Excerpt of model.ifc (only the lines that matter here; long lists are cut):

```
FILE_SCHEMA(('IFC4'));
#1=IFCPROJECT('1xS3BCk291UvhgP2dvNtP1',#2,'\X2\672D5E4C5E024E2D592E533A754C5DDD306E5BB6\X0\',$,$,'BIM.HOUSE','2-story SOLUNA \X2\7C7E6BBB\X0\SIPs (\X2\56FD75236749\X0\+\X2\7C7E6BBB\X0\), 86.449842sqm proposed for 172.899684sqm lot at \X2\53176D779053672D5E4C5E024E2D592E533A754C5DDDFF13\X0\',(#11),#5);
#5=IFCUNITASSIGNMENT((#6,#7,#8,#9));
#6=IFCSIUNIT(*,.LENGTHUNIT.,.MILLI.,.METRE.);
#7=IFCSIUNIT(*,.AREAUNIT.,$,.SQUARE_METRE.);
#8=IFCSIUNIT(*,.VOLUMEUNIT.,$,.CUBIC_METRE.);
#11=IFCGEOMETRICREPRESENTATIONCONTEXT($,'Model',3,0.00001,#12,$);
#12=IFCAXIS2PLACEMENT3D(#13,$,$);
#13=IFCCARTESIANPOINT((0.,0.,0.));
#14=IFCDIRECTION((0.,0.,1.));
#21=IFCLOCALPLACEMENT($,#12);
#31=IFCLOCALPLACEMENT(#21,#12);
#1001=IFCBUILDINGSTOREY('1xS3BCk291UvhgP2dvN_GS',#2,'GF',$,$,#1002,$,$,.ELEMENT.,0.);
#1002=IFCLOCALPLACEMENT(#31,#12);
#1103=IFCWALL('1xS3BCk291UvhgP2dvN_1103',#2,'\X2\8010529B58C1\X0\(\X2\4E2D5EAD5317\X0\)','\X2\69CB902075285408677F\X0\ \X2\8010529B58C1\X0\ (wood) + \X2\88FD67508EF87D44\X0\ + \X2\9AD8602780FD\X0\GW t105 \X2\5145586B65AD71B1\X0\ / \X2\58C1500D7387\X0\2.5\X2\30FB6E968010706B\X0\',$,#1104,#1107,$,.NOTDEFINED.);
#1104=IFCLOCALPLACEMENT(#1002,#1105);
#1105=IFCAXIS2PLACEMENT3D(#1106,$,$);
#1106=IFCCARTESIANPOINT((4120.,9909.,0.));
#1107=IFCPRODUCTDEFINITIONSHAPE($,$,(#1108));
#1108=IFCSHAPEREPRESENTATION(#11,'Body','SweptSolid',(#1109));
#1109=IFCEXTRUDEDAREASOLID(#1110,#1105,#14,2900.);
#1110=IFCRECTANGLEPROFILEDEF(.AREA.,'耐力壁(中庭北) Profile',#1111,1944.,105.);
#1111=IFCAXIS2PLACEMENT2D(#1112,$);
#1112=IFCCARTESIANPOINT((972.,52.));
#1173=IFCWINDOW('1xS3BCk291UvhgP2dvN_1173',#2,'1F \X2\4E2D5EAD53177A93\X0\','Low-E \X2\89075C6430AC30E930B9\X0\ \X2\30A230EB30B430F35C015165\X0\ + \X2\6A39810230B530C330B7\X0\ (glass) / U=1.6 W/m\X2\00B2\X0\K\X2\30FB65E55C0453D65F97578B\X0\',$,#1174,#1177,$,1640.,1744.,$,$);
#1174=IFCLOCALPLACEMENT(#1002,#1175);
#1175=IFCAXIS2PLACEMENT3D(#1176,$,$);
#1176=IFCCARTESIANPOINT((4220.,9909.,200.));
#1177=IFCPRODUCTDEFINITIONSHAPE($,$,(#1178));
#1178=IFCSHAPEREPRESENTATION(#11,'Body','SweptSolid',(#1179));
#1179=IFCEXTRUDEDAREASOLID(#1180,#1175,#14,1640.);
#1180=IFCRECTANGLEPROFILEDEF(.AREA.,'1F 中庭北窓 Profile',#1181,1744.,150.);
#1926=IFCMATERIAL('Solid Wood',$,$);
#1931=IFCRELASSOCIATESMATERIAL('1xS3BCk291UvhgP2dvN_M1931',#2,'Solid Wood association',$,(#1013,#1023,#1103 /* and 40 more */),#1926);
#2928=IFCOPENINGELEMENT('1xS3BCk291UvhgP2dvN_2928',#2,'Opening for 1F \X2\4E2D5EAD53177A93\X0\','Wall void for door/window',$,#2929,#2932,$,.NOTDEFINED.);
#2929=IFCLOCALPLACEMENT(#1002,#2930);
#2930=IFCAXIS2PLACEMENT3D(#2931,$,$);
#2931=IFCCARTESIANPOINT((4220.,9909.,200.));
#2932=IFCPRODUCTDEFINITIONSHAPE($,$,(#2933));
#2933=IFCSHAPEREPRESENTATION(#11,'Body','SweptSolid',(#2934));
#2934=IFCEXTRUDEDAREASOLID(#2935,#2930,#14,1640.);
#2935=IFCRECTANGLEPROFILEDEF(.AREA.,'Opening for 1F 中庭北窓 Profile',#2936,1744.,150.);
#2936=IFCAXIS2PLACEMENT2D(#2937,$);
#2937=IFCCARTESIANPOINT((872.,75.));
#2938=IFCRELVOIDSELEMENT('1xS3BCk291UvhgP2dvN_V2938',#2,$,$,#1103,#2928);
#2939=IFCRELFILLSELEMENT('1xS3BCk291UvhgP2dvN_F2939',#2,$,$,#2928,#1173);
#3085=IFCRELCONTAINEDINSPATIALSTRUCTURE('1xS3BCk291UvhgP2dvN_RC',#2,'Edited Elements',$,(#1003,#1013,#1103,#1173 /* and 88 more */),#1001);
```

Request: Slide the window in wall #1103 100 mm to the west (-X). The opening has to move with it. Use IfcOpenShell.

```python
import ifcopenshell
import ifcopenshell.api.geometry
import ifcopenshell.util.placement

model = ifcopenshell.open("model.ifc")

window = model.by_guid("1xS3BCk291UvhgP2dvN_1173")
opening = window.FillsVoids[0].RelatingOpeningElement
wall = opening.VoidsElements[0].RelatingBuildingElement

wall_matrix = ifcopenshell.util.placement.get_local_placement(wall.ObjectPlacement)
shift = wall_matrix[:3, 0] * -100.0
before = ifcopenshell.util.placement.get_local_placement(window.ObjectPlacement)[:3, 3].copy()

# The window is not placed relative to its opening, so move both.
for product in (opening, window):
    matrix = ifcopenshell.util.placement.get_local_placement(product.ObjectPlacement)
    matrix[:3, 3] += shift
    ifcopenshell.api.geometry.edit_object_placement(model, product=product, matrix=matrix, is_si=False)

after = ifcopenshell.util.placement.get_local_placement(window.ObjectPlacement)[:3, 3]
print("window moved by", (after - before).round(3) + 0.0)

model.write("model_rev.ifc")
```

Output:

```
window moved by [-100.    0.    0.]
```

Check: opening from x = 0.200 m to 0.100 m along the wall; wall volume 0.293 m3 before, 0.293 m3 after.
